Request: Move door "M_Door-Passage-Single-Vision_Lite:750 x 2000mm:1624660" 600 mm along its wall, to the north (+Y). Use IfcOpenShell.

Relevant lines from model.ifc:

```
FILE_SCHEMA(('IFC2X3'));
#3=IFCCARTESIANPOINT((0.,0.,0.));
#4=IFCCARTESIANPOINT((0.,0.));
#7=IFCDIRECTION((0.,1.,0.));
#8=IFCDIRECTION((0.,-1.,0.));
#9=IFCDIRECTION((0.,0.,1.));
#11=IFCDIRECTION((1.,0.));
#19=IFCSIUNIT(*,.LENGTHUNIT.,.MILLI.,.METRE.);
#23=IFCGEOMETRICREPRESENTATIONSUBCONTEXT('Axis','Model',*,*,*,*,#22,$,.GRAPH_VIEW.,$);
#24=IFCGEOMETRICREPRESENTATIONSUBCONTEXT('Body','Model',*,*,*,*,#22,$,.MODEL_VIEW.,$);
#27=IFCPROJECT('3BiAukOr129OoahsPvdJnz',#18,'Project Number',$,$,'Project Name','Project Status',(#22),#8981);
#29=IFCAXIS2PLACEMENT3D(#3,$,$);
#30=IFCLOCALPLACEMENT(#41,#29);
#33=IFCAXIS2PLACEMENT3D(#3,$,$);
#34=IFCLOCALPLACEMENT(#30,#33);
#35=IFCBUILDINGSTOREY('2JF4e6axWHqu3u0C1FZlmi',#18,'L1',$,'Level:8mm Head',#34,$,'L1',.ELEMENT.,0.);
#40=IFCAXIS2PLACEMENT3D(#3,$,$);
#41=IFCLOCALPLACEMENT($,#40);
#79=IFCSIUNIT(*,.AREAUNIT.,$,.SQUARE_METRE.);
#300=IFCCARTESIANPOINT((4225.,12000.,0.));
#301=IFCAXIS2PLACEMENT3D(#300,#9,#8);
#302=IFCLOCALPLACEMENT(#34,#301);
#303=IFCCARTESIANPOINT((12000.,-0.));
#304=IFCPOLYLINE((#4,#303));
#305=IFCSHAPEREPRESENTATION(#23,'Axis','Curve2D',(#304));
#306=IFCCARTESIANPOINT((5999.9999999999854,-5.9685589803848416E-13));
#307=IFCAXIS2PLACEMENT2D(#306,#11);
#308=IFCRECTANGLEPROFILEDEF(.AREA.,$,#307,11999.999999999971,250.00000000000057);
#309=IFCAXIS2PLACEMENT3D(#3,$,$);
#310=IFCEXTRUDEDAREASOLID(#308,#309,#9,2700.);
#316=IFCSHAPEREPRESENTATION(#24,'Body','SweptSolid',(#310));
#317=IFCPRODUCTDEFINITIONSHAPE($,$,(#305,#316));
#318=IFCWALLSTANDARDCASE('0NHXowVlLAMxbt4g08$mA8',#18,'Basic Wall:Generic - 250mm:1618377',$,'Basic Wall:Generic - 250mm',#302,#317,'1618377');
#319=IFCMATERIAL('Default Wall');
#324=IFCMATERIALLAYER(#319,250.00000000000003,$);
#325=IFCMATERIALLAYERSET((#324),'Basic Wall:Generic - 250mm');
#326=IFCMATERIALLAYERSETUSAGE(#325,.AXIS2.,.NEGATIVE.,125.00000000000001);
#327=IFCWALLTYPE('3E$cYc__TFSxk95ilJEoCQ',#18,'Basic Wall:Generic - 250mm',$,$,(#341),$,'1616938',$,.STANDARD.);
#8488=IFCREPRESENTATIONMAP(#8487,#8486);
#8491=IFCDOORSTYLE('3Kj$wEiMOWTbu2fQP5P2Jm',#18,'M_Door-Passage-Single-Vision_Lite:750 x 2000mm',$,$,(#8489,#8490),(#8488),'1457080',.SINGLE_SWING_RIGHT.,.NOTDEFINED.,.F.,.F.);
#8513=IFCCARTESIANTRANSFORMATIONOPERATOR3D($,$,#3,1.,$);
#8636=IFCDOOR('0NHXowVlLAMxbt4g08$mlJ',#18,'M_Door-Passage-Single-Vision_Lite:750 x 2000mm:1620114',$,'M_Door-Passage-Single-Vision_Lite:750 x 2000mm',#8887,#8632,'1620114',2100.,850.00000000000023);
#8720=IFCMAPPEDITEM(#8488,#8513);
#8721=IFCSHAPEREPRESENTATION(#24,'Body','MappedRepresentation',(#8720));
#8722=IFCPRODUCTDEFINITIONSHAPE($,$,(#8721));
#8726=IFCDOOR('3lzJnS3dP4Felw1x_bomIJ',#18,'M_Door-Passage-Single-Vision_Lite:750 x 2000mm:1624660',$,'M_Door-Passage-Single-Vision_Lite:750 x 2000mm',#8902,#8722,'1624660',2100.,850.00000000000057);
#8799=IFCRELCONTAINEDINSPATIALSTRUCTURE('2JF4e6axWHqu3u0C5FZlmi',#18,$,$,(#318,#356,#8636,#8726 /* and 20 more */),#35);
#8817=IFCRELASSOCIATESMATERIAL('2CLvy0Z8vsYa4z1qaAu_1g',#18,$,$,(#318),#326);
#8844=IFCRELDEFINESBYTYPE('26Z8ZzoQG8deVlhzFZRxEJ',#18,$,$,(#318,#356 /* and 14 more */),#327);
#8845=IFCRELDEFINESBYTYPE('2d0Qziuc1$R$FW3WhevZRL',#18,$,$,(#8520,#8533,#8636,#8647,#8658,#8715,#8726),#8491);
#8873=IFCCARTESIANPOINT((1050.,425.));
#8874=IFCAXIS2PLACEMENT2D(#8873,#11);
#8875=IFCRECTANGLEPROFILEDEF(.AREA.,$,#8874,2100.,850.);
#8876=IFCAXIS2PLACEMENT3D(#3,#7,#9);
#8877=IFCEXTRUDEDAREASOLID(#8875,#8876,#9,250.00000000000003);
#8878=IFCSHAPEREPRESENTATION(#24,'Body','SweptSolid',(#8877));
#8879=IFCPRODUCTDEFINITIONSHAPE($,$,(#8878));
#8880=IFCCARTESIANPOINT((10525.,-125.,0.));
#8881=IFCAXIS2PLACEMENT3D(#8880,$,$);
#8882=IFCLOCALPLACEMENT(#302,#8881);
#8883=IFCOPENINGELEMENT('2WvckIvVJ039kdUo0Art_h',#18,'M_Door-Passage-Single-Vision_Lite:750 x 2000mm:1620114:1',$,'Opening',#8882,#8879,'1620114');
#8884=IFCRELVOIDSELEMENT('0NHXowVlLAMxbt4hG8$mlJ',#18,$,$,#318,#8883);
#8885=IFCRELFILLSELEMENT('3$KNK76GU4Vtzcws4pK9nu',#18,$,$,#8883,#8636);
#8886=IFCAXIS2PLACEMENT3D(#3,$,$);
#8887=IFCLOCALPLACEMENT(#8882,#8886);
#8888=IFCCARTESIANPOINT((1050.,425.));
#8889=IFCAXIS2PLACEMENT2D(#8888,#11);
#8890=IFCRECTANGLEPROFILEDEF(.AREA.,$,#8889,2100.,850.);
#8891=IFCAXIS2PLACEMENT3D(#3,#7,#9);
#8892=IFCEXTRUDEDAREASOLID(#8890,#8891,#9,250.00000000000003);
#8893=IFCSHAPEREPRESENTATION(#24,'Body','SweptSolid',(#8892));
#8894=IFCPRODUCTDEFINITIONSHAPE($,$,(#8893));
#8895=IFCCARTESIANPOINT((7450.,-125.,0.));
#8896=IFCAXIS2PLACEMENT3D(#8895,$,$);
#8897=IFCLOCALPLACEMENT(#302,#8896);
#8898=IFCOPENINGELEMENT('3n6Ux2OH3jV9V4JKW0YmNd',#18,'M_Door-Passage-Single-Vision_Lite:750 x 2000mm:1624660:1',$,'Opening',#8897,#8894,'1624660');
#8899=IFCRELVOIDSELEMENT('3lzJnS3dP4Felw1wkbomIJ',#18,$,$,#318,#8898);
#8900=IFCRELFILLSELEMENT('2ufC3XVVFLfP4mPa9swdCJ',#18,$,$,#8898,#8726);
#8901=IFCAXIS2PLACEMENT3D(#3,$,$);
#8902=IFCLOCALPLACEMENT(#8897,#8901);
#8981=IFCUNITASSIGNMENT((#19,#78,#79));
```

```python
import ifcopenshell
import ifcopenshell.api.geometry
import ifcopenshell.util.placement
import ifcopenshell.util.unit

model = ifcopenshell.open("model.ifc")
unit_scale = ifcopenshell.util.unit.calculate_unit_scale(model)

door = model.by_id(8726)
opening = door.FillsVoids[0].RelatingOpeningElement
wall = opening.VoidsElements[0].RelatingBuildingElement

wall_matrix = ifcopenshell.util.placement.get_local_placement(wall.ObjectPlacement)
shift = wall_matrix[:3, 0] * -0.6 / unit_scale
before = ifcopenshell.util.placement.get_local_placement(door.ObjectPlacement)[:3, 3].copy()

# The door is placed relative to its opening, so it follows when the opening moves.
matrix = ifcopenshell.util.placement.get_local_placement(opening.ObjectPlacement)
matrix[:3, 3] += shift
ifcopenshell.api.geometry.edit_object_placement(
    model, product=opening, matrix=matrix, is_si=False, should_transform_children=True
)

after = ifcopenshell.util.placement.get_local_placement(door.ObjectPlacement)[:3, 3]
print("door moved by", (after - before).round(3) + 0.0)

model.write("model_updated.ifc")
```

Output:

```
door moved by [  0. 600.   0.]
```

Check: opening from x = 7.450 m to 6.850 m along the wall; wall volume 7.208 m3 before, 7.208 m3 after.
